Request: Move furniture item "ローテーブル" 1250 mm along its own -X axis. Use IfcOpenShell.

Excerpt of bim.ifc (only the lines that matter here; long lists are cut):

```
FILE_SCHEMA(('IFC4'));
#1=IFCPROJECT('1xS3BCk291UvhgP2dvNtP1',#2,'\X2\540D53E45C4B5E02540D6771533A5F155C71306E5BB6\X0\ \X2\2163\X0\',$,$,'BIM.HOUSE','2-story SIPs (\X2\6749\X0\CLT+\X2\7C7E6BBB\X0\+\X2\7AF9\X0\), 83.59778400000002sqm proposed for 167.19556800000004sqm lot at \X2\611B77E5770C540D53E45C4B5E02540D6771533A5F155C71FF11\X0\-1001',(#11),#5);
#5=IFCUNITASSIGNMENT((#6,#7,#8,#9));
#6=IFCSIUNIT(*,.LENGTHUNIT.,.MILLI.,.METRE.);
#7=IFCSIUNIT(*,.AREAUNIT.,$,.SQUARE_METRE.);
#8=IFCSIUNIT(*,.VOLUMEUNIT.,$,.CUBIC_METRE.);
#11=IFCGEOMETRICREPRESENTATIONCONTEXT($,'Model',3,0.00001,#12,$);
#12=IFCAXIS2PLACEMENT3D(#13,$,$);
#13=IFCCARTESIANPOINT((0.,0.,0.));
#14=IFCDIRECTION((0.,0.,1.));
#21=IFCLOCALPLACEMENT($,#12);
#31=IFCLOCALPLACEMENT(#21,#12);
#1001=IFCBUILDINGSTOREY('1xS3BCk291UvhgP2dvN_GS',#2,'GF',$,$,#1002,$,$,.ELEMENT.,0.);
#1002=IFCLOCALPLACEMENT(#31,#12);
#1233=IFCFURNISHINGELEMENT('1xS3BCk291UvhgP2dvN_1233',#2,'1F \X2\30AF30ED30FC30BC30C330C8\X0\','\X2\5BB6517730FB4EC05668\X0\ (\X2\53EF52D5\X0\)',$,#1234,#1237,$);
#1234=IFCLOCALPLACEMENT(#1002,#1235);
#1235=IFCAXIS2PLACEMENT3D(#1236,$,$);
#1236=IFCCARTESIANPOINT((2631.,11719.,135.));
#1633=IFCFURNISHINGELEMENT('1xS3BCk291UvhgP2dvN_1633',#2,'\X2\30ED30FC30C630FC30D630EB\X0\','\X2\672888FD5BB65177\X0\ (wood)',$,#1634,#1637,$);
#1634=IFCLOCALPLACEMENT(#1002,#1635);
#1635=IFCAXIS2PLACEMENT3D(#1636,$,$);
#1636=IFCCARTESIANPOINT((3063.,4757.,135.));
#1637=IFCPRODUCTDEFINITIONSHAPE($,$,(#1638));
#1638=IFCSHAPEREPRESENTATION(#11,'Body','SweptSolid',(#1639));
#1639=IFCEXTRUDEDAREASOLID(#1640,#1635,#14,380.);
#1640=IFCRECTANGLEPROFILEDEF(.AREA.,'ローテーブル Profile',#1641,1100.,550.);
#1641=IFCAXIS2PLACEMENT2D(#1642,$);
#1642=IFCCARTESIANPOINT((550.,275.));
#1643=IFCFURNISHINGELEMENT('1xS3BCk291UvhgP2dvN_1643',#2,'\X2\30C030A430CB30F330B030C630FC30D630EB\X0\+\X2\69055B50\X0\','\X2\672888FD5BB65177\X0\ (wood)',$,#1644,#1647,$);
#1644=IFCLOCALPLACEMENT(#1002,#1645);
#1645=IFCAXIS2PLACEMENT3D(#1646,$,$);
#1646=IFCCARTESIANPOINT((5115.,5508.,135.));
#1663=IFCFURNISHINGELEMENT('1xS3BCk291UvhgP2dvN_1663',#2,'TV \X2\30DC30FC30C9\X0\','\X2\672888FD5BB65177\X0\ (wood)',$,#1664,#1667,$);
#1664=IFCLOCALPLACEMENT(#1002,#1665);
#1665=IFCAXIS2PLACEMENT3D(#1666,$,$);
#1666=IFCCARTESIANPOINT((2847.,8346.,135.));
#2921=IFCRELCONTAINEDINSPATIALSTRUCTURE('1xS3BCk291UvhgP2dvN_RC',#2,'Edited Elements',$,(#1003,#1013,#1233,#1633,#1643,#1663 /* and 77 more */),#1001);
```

```python
import ifcopenshell
import ifcopenshell.api.geometry
import ifcopenshell.util.placement
import ifcopenshell.util.unit

model = ifcopenshell.open("bim.ifc")
unit_scale = ifcopenshell.util.unit.calculate_unit_scale(model)

item = model.by_guid("1xS3BCk291UvhgP2dvN_1633")
matrix = ifcopenshell.util.placement.get_local_placement(item.ObjectPlacement)
matrix[:3, 3] -= matrix[:3, 0] * 1.25 / unit_scale
ifcopenshell.api.geometry.edit_object_placement(model, product=item, matrix=matrix, is_si=False)

print(ifcopenshell.util.placement.get_local_placement(item.ObjectPlacement).round(3) + 0.0)

model.write("bim_rev.ifc")
```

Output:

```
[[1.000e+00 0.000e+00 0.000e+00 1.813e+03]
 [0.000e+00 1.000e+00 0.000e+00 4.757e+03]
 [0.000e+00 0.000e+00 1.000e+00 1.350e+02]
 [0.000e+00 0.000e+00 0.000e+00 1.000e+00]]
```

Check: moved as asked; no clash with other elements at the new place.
